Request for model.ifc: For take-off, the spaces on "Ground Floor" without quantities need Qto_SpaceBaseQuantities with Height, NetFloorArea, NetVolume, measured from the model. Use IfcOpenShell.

First a look at what the model holds.

```python
import ifcopenshell
import ifcopenshell.util.element
import ifcopenshell.util.unit

model = ifcopenshell.open("model.ifc")
print(model.schema)
for unit_type in ("LENGTHUNIT", "AREAUNIT", "VOLUMEUNIT"):
    print(unit_type, ifcopenshell.util.unit.calculate_unit_scale(model, unit_type))
storey = next(s for s in model.by_type("IfcBuildingStorey") if s.Name == "Ground Floor")
spaces = [e for e in ifcopenshell.util.element.get_decomposition(storey) if e.is_a("IfcSpace")]
for e in sorted(spaces, key=lambda e: e.id()):
    print(e.id(), e.is_a(), e.Name, list(ifcopenshell.util.element.get_psets(e, qtos_only=True)), sep=" | ")
```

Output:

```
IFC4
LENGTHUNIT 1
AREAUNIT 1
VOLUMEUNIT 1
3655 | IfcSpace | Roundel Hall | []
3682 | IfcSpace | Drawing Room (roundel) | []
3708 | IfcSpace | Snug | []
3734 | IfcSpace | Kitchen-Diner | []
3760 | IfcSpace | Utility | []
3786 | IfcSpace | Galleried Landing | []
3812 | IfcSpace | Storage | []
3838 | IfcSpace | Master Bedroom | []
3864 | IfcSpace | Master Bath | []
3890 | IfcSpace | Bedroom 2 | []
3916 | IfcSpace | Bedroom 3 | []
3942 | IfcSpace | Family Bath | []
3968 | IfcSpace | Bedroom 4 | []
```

```python
import ifcopenshell
import ifcopenshell.api.pset
import ifcopenshell.geom
import ifcopenshell.util.element
import ifcopenshell.util.shape
import ifcopenshell.util.unit

model = ifcopenshell.open("model.ifc")
unit_scale = ifcopenshell.util.unit.calculate_unit_scale(model)
area_scale = ifcopenshell.util.unit.calculate_unit_scale(model, "AREAUNIT")
volume_scale = ifcopenshell.util.unit.calculate_unit_scale(model, "VOLUMEUNIT")
settings = ifcopenshell.geom.settings()

storey = next(s for s in model.by_type("IfcBuildingStorey") if s.Name == "Ground Floor")
spaces = [e for e in ifcopenshell.util.element.get_decomposition(storey) if e.is_a("IfcSpace")]

for e in sorted(spaces, key=lambda e: e.id()):
    if ifcopenshell.util.element.get_psets(e, qtos_only=True, should_inherit=False):
        continue
    # Geometry comes back in metres, in the element's own axes.
    shape = ifcopenshell.geom.create_shape(settings, e)
    values = {
        "Height": ifcopenshell.util.shape.get_z(shape.geometry) / unit_scale,
        "NetFloorArea": ifcopenshell.util.shape.get_footprint_area(shape.geometry) / area_scale,
        "NetVolume": ifcopenshell.util.shape.get_volume(shape.geometry) / volume_scale,
    }
    qto = ifcopenshell.api.pset.add_qto(model, product=e, name="Qto_SpaceBaseQuantities")
    ifcopenshell.api.pset.edit_qto(model, qto=qto, properties=values)
    print(e.id(), {k: round(v, 3) for k, v in values.items()})

model.write("model_rev.ifc")
```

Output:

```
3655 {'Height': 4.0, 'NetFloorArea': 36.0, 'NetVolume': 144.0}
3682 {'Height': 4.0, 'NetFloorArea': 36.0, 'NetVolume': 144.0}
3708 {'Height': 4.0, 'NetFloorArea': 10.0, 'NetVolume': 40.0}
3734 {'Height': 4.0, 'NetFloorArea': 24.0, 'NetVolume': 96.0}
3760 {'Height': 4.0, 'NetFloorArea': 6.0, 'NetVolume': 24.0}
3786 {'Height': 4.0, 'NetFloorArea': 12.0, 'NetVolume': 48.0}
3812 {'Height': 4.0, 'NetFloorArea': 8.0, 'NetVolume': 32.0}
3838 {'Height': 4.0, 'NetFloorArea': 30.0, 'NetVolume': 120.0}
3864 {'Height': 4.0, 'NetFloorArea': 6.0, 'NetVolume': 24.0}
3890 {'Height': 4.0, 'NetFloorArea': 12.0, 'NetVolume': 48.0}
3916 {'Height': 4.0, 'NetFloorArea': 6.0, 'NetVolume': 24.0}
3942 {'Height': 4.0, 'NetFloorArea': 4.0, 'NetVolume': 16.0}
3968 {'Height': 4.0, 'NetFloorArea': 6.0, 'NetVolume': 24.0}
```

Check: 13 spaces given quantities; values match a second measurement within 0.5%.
